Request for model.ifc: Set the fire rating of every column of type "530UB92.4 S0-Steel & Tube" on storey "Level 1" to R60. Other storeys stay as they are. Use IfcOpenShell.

First a look at what the model holds.

```python
import ifcopenshell
import ifcopenshell.util.element

model = ifcopenshell.open("model.ifc")
print(model.schema)
storey = next(s for s in model.by_type("IfcBuildingStorey") if s.Name == "Level 1")
columns = [e for e in ifcopenshell.util.element.get_decomposition(storey) if e.is_a("IfcColumn")]
seen = {}
for e in columns:
    element_type = ifcopenshell.util.element.get_type(e)
    key = (element_type.Name if element_type != e and element_type else None, ifcopenshell.util.element.get_pset(e, "Pset_ColumnCommon", "FireRating"))
    seen[key] = seen.get(key, 0) + 1
for (name, value), count in sorted(seen.items(), key=str):
    print(count, "x", name, "|", value)
```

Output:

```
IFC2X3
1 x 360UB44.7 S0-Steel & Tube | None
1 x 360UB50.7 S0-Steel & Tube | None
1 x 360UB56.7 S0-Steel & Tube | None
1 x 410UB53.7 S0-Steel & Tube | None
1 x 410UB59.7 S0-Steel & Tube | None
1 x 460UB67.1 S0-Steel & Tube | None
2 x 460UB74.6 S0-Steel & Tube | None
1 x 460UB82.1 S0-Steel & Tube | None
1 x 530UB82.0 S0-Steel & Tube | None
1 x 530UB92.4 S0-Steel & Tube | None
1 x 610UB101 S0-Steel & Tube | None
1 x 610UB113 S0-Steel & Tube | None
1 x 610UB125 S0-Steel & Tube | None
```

```python
import ifcopenshell
import ifcopenshell.api.pset
import ifcopenshell.util.element

model = ifcopenshell.open("model.ifc")

storey = next(s for s in model.by_type("IfcBuildingStorey") if s.Name == "Level 1")
columns = [e for e in ifcopenshell.util.element.get_decomposition(storey) if e.is_a("IfcColumn")]

count = 0
for e in columns:
    element_type = ifcopenshell.util.element.get_type(e)
    if element_type in (None, e) or element_type.Name != "530UB92.4 S0-Steel & Tube":
        continue
    # add_pset returns the element's existing set when there is one.
    pset = ifcopenshell.api.pset.add_pset(model, product=e, name="Pset_ColumnCommon")
    ifcopenshell.api.pset.edit_pset(model, pset=pset, properties={"FireRating": "R60"})
    count += 1

print(count, "columns updated")

model.write("model_edited.ifc")
```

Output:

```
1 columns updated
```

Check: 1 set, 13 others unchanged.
